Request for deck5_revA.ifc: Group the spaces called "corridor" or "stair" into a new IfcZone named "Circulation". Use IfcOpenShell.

First a look at what the model holds.

```python
import ifcopenshell

model = ifcopenshell.open("deck5_revA.ifc")
print(model.schema)
seen = {}
for space in model.by_type("IfcSpace"):
    seen[space.LongName] = seen.get(space.LongName, 0) + 1
for name, count in sorted(seen.items(), key=str):
    print(count, "x", name)
print("zones:", [z.Name for z in model.by_type("IfcZone")][:20])
```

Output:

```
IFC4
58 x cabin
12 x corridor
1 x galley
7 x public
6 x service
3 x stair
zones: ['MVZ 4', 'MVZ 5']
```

```python
import ifcopenshell
import ifcopenshell.api.group
import ifcopenshell.api.root

model = ifcopenshell.open("deck5_revA.ifc")

names = {"corridor", "stair"}
spaces = [s for s in model.by_type("IfcSpace") if s.LongName in names]

zone = ifcopenshell.api.root.create_entity(model, ifc_class="IfcZone", name="Circulation")
ifcopenshell.api.group.assign_group(model, products=spaces, group=zone)
print(len(spaces), "spaces in", zone.Name)

model.write("deck5_revA_updated.ifc")
```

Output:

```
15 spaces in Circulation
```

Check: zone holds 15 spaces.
